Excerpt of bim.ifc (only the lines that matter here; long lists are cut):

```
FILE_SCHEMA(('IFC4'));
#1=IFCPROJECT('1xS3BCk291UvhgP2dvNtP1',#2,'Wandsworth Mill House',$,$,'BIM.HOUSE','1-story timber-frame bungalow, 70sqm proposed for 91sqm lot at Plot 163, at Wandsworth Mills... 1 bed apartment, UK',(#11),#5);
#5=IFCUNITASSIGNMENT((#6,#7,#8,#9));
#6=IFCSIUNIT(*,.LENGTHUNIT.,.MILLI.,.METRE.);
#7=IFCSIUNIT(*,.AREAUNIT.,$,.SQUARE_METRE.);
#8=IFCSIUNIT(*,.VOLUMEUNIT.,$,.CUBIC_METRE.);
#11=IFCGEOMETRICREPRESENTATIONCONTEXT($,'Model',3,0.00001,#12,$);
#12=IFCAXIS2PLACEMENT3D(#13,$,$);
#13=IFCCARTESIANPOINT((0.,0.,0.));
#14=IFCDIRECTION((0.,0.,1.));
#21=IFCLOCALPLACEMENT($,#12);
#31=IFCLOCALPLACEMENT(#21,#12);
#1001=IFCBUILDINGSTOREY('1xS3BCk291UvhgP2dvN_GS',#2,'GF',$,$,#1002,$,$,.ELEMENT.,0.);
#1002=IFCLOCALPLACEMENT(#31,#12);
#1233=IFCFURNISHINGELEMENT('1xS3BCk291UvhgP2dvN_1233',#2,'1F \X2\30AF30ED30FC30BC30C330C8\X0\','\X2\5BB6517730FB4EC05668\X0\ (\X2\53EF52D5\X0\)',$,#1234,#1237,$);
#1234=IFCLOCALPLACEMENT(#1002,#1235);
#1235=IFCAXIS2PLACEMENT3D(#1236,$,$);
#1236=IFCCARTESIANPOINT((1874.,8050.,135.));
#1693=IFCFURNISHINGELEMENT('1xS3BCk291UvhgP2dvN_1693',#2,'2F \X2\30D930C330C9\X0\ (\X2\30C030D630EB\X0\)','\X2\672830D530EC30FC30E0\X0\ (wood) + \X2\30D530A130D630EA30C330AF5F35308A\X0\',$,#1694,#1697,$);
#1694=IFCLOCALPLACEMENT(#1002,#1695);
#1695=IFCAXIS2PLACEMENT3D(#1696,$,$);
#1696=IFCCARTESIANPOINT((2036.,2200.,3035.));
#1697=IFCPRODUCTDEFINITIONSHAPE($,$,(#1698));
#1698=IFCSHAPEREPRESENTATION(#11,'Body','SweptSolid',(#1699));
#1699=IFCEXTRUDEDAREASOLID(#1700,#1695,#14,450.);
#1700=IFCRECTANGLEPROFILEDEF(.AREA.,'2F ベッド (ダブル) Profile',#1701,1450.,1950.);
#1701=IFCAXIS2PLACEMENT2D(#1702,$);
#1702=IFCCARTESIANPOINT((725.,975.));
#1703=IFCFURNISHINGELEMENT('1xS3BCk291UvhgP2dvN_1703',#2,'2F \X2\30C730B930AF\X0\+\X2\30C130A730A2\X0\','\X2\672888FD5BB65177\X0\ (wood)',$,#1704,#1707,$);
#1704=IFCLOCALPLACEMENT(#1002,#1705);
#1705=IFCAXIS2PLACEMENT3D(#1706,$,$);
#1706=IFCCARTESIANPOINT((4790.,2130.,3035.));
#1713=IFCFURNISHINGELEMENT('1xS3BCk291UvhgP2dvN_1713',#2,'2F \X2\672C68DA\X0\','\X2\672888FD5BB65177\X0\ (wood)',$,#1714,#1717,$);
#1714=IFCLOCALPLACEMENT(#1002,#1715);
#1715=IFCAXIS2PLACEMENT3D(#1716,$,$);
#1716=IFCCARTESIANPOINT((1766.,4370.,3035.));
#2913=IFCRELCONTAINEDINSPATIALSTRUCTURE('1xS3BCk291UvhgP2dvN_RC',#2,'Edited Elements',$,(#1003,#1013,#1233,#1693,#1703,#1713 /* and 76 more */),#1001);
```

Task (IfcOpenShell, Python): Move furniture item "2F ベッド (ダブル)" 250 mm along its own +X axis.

```python
import ifcopenshell
import ifcopenshell.api.geometry
import ifcopenshell.util.placement
import ifcopenshell.util.unit

model = ifcopenshell.open("bim.ifc")
unit_scale = ifcopenshell.util.unit.calculate_unit_scale(model)

item = model.by_guid("1xS3BCk291UvhgP2dvN_1693")
matrix = ifcopenshell.util.placement.get_local_placement(item.ObjectPlacement)
matrix[:3, 3] += matrix[:3, 0] * 0.25 / unit_scale
ifcopenshell.api.geometry.edit_object_placement(model, product=item, matrix=matrix, is_si=False)

print(ifcopenshell.util.placement.get_local_placement(item.ObjectPlacement).round(3) + 0.0)

model.write("bim-out.ifc")
```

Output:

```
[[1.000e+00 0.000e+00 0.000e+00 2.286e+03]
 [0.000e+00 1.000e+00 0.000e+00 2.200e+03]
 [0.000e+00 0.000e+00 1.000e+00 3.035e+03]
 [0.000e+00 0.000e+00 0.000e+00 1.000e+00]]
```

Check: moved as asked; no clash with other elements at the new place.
